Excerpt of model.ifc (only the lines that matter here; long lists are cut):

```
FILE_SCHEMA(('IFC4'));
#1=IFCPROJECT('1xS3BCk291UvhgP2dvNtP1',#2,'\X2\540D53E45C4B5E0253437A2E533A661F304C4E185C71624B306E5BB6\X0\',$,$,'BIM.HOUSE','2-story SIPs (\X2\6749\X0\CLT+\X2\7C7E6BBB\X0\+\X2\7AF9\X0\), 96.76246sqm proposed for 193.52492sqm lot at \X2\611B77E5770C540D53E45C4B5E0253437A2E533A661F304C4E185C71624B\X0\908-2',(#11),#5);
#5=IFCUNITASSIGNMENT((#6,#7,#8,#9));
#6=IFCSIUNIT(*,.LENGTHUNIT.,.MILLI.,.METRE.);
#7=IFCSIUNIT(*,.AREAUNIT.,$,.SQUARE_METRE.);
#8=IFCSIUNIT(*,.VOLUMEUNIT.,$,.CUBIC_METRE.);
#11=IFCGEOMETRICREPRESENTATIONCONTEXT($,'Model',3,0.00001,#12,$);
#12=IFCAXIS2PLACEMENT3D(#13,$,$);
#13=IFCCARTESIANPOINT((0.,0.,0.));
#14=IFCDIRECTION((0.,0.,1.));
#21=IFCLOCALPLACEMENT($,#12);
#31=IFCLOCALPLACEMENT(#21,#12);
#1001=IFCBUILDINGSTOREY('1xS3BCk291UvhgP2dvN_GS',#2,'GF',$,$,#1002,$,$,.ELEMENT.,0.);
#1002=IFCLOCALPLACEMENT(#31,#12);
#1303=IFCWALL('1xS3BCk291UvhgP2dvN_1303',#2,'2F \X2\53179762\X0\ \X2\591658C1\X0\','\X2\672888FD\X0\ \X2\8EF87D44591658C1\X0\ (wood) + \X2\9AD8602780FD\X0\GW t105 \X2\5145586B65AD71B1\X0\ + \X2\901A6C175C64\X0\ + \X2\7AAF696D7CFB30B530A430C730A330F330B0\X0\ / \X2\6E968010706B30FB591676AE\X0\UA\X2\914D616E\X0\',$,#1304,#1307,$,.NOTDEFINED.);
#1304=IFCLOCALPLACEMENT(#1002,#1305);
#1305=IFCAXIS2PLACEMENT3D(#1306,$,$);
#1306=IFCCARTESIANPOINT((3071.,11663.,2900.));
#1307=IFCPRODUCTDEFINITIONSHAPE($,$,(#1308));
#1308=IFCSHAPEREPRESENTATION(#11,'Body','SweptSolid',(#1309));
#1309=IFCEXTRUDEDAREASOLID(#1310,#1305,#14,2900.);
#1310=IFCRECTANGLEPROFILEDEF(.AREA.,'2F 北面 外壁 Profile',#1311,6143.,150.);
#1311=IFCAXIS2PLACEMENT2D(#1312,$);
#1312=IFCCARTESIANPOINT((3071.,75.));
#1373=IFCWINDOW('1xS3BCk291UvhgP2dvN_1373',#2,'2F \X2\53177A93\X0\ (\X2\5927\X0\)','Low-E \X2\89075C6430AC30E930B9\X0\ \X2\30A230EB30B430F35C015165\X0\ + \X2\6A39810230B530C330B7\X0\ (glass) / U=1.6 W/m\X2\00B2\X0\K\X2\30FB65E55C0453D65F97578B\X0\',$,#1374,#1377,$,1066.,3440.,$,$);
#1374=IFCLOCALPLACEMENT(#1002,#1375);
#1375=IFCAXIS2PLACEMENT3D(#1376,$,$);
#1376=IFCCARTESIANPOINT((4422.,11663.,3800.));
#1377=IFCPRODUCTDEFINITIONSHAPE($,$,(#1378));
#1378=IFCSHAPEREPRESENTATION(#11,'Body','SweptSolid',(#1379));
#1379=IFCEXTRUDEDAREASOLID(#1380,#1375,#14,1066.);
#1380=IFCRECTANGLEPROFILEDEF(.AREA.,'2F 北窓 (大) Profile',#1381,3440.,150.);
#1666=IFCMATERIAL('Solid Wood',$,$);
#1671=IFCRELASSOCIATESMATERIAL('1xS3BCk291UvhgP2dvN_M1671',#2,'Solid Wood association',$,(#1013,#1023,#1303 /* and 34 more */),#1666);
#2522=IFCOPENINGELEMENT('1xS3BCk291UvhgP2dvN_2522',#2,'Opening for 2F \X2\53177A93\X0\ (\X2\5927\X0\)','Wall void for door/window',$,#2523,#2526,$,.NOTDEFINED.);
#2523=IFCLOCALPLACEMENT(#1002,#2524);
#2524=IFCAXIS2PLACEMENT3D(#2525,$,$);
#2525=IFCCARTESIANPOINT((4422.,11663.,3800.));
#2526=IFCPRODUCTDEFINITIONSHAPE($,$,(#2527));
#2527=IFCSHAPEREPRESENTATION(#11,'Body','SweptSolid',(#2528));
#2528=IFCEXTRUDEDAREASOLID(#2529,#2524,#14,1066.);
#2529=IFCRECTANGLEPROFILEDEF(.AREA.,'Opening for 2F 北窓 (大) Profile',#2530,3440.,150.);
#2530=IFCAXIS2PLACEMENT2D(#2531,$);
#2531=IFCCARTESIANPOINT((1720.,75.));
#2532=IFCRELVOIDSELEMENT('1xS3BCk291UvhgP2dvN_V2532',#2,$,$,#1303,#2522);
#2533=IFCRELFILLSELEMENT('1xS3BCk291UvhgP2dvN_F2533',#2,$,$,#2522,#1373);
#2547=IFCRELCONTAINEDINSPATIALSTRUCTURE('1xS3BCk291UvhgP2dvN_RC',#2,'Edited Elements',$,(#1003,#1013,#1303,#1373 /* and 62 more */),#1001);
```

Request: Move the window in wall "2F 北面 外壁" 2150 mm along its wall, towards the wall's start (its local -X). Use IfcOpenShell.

```python
import ifcopenshell
import ifcopenshell.api.geometry
import ifcopenshell.util.placement
import ifcopenshell.util.unit

model = ifcopenshell.open("model.ifc")
unit_scale = ifcopenshell.util.unit.calculate_unit_scale(model)

window = model.by_id(1373)
opening = window.FillsVoids[0].RelatingOpeningElement
wall = opening.VoidsElements[0].RelatingBuildingElement

wall_matrix = ifcopenshell.util.placement.get_local_placement(wall.ObjectPlacement)
shift = wall_matrix[:3, 0] * -2.15 / unit_scale
before = ifcopenshell.util.placement.get_local_placement(window.ObjectPlacement)[:3, 3].copy()

# The window is not placed relative to its opening, so move both.
for product in (opening, window):
    matrix = ifcopenshell.util.placement.get_local_placement(product.ObjectPlacement)
    matrix[:3, 3] += shift
    ifcopenshell.api.geometry.edit_object_placement(model, product=product, matrix=matrix, is_si=False)

after = ifcopenshell.util.placement.get_local_placement(window.ObjectPlacement)[:3, 3]
print("window moved by", (after - before).round(3) + 0.0)

model.write("model_updated.ifc")
```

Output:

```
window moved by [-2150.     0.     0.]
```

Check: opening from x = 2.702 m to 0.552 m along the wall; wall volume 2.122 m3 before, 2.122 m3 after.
